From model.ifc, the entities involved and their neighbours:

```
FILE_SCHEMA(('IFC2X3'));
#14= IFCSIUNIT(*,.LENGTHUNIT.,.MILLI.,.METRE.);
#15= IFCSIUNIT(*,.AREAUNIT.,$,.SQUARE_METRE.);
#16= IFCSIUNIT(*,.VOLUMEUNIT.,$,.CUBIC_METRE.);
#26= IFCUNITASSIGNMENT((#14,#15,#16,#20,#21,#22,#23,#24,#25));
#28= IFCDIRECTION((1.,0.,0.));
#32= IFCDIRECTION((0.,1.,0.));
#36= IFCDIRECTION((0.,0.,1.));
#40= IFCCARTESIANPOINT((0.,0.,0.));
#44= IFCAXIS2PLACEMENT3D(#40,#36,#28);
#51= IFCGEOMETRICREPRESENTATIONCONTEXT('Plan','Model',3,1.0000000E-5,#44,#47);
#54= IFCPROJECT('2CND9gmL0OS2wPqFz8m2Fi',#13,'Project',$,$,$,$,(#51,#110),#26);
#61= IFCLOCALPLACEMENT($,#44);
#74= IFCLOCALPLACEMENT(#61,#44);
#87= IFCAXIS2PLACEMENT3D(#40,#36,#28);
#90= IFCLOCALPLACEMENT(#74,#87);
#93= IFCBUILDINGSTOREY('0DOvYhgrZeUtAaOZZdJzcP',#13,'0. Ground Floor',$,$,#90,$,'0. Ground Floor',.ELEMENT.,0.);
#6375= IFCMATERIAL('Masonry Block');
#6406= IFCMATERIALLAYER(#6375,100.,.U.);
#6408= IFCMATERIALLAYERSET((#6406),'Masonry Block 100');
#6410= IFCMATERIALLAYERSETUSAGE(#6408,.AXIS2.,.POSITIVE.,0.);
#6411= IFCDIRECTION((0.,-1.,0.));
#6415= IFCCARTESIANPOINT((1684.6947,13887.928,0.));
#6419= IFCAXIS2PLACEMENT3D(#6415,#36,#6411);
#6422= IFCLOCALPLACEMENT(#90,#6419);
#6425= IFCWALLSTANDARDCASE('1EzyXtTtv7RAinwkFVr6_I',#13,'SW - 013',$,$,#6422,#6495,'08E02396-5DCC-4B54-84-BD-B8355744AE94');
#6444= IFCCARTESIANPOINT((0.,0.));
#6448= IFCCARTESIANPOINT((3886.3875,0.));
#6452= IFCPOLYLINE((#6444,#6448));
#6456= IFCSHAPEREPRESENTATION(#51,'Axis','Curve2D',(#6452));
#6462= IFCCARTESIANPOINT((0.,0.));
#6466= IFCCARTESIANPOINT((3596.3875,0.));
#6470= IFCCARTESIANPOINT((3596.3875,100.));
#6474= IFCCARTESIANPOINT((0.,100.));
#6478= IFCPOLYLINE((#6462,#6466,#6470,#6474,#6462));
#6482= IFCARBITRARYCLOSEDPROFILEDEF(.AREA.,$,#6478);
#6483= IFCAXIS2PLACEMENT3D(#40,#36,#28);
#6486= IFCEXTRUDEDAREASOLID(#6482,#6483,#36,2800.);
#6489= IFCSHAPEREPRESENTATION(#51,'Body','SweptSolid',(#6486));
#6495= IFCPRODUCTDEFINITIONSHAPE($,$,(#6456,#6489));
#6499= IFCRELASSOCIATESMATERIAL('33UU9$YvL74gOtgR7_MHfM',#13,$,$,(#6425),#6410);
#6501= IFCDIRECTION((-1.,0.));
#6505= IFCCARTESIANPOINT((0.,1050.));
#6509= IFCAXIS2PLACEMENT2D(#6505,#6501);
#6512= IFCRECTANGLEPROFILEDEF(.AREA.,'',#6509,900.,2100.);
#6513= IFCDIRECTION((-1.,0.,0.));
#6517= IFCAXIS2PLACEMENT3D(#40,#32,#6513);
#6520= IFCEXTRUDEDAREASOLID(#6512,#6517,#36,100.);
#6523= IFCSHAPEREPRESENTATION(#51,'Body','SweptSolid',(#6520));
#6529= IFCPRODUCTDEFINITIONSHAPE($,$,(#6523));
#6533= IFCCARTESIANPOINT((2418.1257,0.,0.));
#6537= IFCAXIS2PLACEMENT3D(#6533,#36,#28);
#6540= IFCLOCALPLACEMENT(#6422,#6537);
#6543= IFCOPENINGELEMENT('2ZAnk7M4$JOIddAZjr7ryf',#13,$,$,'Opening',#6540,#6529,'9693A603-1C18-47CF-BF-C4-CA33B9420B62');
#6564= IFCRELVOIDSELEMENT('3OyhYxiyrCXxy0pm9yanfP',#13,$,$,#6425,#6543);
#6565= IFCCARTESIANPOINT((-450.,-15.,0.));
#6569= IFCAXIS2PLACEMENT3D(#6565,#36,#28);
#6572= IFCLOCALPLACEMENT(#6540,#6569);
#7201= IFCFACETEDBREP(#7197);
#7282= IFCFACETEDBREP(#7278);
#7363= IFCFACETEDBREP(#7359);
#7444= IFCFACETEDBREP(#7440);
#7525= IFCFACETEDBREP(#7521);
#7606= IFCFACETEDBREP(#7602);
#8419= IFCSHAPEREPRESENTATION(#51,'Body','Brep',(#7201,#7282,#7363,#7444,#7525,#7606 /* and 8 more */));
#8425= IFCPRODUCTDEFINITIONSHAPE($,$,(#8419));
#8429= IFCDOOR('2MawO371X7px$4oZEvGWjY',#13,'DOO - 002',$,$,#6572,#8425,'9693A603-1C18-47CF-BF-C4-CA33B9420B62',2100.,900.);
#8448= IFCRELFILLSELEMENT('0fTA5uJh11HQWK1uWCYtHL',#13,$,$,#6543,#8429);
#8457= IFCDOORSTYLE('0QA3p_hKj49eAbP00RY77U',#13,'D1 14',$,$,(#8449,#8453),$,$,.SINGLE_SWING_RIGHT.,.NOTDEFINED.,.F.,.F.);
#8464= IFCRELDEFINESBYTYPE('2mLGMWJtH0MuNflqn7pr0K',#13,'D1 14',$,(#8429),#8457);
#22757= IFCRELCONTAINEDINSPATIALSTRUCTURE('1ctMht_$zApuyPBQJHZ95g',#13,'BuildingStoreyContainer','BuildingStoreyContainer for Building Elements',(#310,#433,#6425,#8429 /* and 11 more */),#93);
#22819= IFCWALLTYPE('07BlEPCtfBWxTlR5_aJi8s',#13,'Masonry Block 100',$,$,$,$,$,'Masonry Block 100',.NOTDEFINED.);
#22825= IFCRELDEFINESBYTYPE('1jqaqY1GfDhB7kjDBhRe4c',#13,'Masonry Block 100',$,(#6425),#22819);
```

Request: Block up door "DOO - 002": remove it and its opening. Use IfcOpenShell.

```python
import ifcopenshell
import ifcopenshell.api.feature
import ifcopenshell.api.root
import ifcopenshell.geom
import ifcopenshell.util.shape

model = ifcopenshell.open("model.ifc")
settings = ifcopenshell.geom.settings()


def volume(element):
    """Net volume in cubic metres, openings subtracted."""
    shape = ifcopenshell.geom.create_shape(settings, element)
    return ifcopenshell.util.shape.get_volume(shape.geometry)


door = model.by_guid("2MawO371X7px$4oZEvGWjY")
opening = door.FillsVoids[0].RelatingOpeningElement
wall = opening.VoidsElements[0].RelatingBuildingElement
before = volume(wall)

ifcopenshell.api.root.remove_product(model, product=door)
ifcopenshell.api.feature.remove_feature(model, feature=opening)

after = volume(wall)

print(f"wall volume {before:.3f} -> {after:.3f} m3")

model.write("model_updated.ifc")
```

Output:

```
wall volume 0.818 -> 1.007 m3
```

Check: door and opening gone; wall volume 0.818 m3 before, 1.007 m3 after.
